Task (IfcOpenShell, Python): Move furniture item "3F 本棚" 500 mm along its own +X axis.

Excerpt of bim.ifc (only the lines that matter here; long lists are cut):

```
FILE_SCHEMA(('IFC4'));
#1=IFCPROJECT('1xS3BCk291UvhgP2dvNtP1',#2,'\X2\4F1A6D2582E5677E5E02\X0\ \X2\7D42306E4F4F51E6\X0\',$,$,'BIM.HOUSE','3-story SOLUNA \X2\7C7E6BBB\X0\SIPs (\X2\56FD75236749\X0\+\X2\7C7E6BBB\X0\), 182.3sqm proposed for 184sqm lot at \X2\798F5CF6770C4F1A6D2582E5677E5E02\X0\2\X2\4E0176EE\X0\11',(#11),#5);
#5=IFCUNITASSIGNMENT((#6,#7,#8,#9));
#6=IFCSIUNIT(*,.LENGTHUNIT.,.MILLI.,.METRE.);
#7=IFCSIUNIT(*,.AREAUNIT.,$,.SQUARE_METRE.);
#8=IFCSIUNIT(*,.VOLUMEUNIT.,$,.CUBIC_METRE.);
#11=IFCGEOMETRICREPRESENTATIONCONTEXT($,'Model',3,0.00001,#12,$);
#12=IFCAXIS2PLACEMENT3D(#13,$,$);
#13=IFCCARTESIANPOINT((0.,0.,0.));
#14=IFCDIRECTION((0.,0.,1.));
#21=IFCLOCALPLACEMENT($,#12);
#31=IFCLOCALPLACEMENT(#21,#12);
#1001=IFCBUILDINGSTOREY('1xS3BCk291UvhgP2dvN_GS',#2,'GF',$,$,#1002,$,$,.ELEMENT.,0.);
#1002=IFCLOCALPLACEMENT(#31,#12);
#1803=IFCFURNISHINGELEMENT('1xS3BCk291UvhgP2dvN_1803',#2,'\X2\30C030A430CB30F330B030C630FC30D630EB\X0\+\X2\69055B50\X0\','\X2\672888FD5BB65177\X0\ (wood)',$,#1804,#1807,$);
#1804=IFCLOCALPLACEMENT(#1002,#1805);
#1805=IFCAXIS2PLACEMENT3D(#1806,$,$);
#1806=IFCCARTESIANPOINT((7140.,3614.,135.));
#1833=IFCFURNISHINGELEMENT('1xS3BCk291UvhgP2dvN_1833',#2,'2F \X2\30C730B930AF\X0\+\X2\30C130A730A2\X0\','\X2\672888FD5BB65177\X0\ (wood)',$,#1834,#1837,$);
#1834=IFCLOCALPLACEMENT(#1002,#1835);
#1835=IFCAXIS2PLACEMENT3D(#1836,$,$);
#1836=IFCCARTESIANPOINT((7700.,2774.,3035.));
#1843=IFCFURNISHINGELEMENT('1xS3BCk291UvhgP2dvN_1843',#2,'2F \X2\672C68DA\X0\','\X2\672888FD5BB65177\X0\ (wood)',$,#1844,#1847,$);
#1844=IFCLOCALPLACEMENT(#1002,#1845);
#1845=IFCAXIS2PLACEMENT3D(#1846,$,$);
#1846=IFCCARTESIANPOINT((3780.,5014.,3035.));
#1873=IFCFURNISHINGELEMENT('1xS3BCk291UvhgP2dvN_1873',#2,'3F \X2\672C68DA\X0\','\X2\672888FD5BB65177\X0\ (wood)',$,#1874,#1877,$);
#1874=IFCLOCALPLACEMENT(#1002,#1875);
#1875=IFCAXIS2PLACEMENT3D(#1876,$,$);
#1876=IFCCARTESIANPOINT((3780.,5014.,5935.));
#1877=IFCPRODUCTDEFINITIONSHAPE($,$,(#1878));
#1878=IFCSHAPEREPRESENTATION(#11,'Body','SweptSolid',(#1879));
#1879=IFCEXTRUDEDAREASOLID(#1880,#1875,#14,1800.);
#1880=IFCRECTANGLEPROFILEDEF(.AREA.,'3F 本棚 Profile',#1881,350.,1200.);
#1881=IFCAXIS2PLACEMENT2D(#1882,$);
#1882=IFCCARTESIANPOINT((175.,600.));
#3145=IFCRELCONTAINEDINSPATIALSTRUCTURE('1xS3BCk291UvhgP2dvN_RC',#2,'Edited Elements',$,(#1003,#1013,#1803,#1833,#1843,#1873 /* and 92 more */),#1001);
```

```python
import ifcopenshell
import ifcopenshell.api.geometry
import ifcopenshell.util.placement

model = ifcopenshell.open("bim.ifc")

item = model.by_id(1873)
matrix = ifcopenshell.util.placement.get_local_placement(item.ObjectPlacement)
matrix[:3, 3] += matrix[:3, 0] * 500.0
ifcopenshell.api.geometry.edit_object_placement(model, product=item, matrix=matrix, is_si=False)

print(ifcopenshell.util.placement.get_local_placement(item.ObjectPlacement).round(3) + 0.0)

model.write("bim_v2.ifc")
```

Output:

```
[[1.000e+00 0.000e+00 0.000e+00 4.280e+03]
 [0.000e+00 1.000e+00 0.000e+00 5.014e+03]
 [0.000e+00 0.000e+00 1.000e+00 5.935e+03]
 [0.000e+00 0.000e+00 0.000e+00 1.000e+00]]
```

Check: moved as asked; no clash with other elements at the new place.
